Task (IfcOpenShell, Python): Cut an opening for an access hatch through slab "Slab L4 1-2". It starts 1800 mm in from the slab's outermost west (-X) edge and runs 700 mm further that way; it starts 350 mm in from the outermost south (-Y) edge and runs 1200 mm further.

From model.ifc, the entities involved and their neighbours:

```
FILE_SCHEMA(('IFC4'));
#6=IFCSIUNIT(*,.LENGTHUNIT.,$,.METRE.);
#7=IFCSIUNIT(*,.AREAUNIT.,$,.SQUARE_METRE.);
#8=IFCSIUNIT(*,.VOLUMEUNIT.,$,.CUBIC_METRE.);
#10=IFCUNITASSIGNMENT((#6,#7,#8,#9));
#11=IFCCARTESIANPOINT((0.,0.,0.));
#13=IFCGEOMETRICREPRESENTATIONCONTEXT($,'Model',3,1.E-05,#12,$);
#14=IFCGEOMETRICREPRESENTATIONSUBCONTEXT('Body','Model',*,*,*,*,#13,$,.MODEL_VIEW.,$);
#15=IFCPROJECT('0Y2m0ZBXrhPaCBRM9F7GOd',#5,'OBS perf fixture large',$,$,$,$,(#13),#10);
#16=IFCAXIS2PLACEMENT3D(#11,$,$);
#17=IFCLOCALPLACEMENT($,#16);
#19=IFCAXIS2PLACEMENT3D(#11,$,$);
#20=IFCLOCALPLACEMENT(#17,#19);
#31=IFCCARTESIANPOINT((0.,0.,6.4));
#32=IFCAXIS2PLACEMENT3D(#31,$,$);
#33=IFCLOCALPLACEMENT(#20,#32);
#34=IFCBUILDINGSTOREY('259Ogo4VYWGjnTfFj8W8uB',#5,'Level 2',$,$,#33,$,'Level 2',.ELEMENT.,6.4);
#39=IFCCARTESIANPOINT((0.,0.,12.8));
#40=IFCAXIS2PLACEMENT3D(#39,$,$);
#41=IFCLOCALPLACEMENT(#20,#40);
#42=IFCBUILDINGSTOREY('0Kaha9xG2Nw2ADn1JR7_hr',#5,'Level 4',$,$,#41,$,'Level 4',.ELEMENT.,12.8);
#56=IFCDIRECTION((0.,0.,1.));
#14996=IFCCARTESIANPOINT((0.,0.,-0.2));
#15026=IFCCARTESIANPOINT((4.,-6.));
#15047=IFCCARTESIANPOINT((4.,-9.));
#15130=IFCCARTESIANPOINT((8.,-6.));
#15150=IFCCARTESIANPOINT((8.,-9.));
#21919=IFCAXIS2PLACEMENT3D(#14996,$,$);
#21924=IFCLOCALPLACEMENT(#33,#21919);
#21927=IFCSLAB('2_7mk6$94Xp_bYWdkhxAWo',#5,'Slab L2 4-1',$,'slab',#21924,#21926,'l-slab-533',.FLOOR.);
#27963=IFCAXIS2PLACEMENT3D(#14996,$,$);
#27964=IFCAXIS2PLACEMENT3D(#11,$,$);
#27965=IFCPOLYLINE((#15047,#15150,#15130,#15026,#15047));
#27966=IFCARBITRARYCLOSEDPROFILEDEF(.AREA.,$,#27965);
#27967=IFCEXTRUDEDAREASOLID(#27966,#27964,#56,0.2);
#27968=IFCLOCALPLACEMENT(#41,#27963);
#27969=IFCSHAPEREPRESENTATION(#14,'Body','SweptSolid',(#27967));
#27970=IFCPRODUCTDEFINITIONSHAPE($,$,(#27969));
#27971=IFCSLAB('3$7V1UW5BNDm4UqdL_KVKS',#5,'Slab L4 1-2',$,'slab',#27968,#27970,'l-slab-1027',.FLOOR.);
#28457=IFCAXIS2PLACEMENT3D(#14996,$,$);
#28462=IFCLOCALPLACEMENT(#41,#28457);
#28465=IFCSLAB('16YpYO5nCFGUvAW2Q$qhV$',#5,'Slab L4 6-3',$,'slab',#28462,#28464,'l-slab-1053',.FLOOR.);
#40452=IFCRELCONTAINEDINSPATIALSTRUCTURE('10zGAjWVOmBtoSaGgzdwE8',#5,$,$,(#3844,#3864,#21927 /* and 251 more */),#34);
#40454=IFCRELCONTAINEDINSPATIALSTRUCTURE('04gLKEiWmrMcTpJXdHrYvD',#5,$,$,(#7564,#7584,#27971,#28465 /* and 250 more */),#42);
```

```python
import numpy as np
import ifcopenshell
import ifcopenshell.api.feature
import ifcopenshell.api.geometry
import ifcopenshell.api.root
import ifcopenshell.geom
import ifcopenshell.util.placement
import ifcopenshell.util.representation
import ifcopenshell.util.shape
import ifcopenshell.util.unit

model = ifcopenshell.open("model.ifc")
unit_scale = ifcopenshell.util.unit.calculate_unit_scale(model)
settings = ifcopenshell.geom.settings()


def volume(element):
    """Net volume in cubic metres, openings subtracted."""
    shape = ifcopenshell.geom.create_shape(settings, element)
    return ifcopenshell.util.shape.get_volume(shape.geometry)


slab = model.by_guid("3$7V1UW5BNDm4UqdL_KVKS")
before = volume(slab)

# Extent in the slab's own axes, in metres. The edges named are its -X and -Y sides.
slab_shape = ifcopenshell.geom.create_shape(settings, slab)
vertices = ifcopenshell.util.shape.get_vertices(slab_shape.geometry)
x_min, y_min, bottom = vertices.min(axis=0)
top = vertices[:, 2].max()

opening = ifcopenshell.api.root.create_entity(model, ifc_class="IfcOpeningElement", name="Access hatch opening", predefined_type="OPENING")
context = ifcopenshell.util.representation.get_context(model, "Model", "Body", "MODEL_VIEW")
width, depth = 0.7, 1.2
outline = [(0.0, 0.0), (width, 0.0), (width, depth), (0.0, depth), (0.0, 0.0)]
# Overshoot both faces by 50 mm so the cut is clean.
shape = ifcopenshell.api.geometry.add_slab_representation(
    model, context=context, depth=top - bottom + 0.1, polyline=outline
)
ifcopenshell.api.geometry.assign_representation(model, product=opening, representation=shape)

matrix = ifcopenshell.util.placement.get_local_placement(slab.ObjectPlacement)
matrix[:, 3] = matrix @ np.append(np.array([x_min + 1.8, y_min + 0.35, bottom - 0.05]) / unit_scale, 1.0)
ifcopenshell.api.geometry.edit_object_placement(model, product=opening, matrix=matrix, is_si=False)
ifcopenshell.api.feature.add_feature(model, feature=opening, element=slab)

after = volume(slab)

print(f"slab volume {before:.3f} -> {after:.3f} m3")

model.write("model_rev.ifc")
```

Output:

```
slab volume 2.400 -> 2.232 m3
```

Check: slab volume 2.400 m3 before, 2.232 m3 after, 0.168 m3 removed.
